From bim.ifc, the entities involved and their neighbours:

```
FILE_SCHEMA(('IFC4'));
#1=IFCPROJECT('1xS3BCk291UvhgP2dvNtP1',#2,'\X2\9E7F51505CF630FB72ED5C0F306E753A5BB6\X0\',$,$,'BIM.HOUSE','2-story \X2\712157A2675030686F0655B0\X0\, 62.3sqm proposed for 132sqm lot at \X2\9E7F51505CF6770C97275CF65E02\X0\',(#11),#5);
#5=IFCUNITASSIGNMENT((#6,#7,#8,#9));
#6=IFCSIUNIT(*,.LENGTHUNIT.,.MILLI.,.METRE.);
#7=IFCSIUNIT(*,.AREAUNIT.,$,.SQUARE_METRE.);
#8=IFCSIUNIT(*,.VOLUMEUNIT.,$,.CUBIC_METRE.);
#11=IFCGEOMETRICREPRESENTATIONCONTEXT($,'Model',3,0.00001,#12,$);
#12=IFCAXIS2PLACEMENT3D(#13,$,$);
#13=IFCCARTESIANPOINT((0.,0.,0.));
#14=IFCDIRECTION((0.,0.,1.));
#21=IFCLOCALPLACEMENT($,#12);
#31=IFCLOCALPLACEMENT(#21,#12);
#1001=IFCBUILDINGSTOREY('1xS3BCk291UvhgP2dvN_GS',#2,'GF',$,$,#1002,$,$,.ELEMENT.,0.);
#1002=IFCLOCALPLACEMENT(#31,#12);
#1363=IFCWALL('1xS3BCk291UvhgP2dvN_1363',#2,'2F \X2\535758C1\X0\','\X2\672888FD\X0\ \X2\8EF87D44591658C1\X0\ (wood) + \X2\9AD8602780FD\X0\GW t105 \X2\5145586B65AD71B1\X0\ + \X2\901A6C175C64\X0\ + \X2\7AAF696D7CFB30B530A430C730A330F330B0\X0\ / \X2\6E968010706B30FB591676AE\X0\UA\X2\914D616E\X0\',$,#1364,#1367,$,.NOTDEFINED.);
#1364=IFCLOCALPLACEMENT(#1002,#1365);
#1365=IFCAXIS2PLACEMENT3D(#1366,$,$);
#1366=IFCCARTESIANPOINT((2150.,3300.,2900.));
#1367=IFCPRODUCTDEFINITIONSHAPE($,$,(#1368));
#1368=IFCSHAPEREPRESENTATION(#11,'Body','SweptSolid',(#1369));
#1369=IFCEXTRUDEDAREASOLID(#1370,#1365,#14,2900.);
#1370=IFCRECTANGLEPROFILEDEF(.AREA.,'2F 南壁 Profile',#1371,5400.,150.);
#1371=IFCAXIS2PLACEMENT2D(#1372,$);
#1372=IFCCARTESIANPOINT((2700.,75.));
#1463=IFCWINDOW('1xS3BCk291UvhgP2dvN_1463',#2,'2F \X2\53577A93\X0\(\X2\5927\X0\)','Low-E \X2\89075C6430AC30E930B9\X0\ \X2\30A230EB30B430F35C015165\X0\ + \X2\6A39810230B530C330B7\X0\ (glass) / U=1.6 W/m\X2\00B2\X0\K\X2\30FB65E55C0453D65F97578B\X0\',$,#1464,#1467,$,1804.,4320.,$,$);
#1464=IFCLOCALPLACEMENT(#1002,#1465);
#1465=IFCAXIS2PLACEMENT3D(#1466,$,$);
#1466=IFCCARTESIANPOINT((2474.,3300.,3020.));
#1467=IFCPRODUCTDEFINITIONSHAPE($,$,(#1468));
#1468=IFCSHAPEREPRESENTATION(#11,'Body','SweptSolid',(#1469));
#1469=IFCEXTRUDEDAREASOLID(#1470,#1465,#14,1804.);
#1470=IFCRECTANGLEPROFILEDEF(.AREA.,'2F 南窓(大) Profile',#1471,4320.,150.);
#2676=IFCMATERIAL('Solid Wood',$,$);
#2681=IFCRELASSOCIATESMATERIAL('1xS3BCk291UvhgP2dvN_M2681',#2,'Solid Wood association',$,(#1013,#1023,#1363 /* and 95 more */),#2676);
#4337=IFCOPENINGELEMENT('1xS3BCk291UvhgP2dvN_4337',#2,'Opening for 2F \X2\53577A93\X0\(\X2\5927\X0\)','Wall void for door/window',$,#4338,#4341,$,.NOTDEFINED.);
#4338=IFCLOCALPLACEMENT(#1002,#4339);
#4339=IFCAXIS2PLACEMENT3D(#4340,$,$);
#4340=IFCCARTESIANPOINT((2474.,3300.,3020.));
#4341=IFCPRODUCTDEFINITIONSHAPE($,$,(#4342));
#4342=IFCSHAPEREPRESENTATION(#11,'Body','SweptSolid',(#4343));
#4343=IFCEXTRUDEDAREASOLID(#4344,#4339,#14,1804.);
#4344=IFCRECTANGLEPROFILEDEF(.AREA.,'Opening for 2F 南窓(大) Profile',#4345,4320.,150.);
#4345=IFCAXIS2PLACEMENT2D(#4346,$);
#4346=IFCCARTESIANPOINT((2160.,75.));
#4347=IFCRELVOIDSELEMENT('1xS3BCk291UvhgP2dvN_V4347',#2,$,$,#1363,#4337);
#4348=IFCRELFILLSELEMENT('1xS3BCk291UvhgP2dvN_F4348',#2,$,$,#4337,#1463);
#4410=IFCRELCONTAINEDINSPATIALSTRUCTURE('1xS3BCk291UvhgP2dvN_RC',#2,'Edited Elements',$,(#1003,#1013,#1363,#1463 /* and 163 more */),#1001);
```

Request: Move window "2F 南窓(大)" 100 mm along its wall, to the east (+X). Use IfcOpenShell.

```python
import ifcopenshell
import ifcopenshell.api.geometry
import ifcopenshell.util.placement

model = ifcopenshell.open("bim.ifc")

window = model.by_id(1463)
opening = window.FillsVoids[0].RelatingOpeningElement
wall = opening.VoidsElements[0].RelatingBuildingElement

wall_matrix = ifcopenshell.util.placement.get_local_placement(wall.ObjectPlacement)
shift = wall_matrix[:3, 0] * 100.0
before = ifcopenshell.util.placement.get_local_placement(window.ObjectPlacement)[:3, 3].copy()

# The window is not placed relative to its opening, so move both.
for product in (opening, window):
    matrix = ifcopenshell.util.placement.get_local_placement(product.ObjectPlacement)
    matrix[:3, 3] += shift
    ifcopenshell.api.geometry.edit_object_placement(model, product=product, matrix=matrix, is_si=False)

after = ifcopenshell.util.placement.get_local_placement(window.ObjectPlacement)[:3, 3]
print("window moved by", (after - before).round(3) + 0.0)

model.write("bim-out.ifc")
```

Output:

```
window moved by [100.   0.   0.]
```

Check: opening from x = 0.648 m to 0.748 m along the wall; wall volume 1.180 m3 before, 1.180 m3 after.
